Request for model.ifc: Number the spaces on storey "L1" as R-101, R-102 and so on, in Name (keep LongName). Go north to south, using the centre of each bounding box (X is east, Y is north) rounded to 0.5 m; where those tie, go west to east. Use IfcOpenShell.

First a look at what the model holds.

```python
import ifcopenshell
import ifcopenshell.util.element
import ifcopenshell.util.placement

model = ifcopenshell.open("model.ifc")
print(model.schema)
storey = next(s for s in model.by_type("IfcBuildingStorey") if s.Name == "L1")
spaces = [e for e in ifcopenshell.util.element.get_decomposition(storey) if e.is_a("IfcSpace")]
for e in sorted(spaces, key=lambda e: e.id()):
    origin = ifcopenshell.util.placement.get_local_placement(e.ObjectPlacement)[:3, 3]
    print(e.id(), e.Name, e.LongName, origin.round(2) + 0.0, sep=" | ")
```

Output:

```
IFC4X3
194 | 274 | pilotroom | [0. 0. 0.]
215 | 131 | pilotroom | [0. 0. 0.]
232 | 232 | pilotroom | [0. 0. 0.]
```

```python
import ifcopenshell
import ifcopenshell.geom
import ifcopenshell.util.element
import ifcopenshell.util.shape

model = ifcopenshell.open("model.ifc")
settings = ifcopenshell.geom.settings()
settings.set("use-world-coords", True)


def centre(element):
    shape = ifcopenshell.geom.create_shape(settings, element)
    return ifcopenshell.util.shape.get_bbox_centroid(shape.geometry)


storey = next(s for s in model.by_type("IfcBuildingStorey") if s.Name == "L1")
spaces = [e for e in ifcopenshell.util.element.get_decomposition(storey) if e.is_a("IfcSpace")]

# Insertion points can sit at a corner or the storey origin, so sort by the geometry (in metres).
centres = {e: centre(e) for e in spaces}
spaces.sort(key=lambda e: (-round(centres[e][1] / 0.5), centres[e][0]))

for i, e in enumerate(spaces, start=1):
    number = f"R-1{i:02d}"
    e.Name = number
    print(e.id(), number)

model.write("model_edited.ifc")
```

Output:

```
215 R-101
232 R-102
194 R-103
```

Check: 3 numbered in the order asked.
